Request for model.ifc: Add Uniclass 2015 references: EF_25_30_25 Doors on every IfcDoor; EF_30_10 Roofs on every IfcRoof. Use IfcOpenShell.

First a look at what the model holds.

```python
import ifcopenshell

model = ifcopenshell.open("model.ifc")
print(model.schema)
print("classifications:", [c.Name for c in model.by_type("IfcClassification")])
for ifc_class in ("IfcDoor", "IfcRoof", "IfcStair", "IfcWall", "IfcWindow"):
    print(ifc_class, len(model.by_type(ifc_class)))
```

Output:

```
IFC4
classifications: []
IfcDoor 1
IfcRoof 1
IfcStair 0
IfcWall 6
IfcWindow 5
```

```python
import ifcopenshell
import ifcopenshell.api.classification

model = ifcopenshell.open("model.ifc")

system = ifcopenshell.api.classification.add_classification(model, classification="Uniclass 2015")

codes = {
    "IfcDoor": ("EF_25_30_25", "Doors"),
    "IfcRoof": ("EF_30_10", "Roofs"),
}
for ifc_class, (code, name) in codes.items():
    products = model.by_type(ifc_class)
    ifcopenshell.api.classification.add_reference(
        model, products=products, classification=system, identification=code, name=name
    )
    print(code, len(products))

model.write("model_rev.ifc")
```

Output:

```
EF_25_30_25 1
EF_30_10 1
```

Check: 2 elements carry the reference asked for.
